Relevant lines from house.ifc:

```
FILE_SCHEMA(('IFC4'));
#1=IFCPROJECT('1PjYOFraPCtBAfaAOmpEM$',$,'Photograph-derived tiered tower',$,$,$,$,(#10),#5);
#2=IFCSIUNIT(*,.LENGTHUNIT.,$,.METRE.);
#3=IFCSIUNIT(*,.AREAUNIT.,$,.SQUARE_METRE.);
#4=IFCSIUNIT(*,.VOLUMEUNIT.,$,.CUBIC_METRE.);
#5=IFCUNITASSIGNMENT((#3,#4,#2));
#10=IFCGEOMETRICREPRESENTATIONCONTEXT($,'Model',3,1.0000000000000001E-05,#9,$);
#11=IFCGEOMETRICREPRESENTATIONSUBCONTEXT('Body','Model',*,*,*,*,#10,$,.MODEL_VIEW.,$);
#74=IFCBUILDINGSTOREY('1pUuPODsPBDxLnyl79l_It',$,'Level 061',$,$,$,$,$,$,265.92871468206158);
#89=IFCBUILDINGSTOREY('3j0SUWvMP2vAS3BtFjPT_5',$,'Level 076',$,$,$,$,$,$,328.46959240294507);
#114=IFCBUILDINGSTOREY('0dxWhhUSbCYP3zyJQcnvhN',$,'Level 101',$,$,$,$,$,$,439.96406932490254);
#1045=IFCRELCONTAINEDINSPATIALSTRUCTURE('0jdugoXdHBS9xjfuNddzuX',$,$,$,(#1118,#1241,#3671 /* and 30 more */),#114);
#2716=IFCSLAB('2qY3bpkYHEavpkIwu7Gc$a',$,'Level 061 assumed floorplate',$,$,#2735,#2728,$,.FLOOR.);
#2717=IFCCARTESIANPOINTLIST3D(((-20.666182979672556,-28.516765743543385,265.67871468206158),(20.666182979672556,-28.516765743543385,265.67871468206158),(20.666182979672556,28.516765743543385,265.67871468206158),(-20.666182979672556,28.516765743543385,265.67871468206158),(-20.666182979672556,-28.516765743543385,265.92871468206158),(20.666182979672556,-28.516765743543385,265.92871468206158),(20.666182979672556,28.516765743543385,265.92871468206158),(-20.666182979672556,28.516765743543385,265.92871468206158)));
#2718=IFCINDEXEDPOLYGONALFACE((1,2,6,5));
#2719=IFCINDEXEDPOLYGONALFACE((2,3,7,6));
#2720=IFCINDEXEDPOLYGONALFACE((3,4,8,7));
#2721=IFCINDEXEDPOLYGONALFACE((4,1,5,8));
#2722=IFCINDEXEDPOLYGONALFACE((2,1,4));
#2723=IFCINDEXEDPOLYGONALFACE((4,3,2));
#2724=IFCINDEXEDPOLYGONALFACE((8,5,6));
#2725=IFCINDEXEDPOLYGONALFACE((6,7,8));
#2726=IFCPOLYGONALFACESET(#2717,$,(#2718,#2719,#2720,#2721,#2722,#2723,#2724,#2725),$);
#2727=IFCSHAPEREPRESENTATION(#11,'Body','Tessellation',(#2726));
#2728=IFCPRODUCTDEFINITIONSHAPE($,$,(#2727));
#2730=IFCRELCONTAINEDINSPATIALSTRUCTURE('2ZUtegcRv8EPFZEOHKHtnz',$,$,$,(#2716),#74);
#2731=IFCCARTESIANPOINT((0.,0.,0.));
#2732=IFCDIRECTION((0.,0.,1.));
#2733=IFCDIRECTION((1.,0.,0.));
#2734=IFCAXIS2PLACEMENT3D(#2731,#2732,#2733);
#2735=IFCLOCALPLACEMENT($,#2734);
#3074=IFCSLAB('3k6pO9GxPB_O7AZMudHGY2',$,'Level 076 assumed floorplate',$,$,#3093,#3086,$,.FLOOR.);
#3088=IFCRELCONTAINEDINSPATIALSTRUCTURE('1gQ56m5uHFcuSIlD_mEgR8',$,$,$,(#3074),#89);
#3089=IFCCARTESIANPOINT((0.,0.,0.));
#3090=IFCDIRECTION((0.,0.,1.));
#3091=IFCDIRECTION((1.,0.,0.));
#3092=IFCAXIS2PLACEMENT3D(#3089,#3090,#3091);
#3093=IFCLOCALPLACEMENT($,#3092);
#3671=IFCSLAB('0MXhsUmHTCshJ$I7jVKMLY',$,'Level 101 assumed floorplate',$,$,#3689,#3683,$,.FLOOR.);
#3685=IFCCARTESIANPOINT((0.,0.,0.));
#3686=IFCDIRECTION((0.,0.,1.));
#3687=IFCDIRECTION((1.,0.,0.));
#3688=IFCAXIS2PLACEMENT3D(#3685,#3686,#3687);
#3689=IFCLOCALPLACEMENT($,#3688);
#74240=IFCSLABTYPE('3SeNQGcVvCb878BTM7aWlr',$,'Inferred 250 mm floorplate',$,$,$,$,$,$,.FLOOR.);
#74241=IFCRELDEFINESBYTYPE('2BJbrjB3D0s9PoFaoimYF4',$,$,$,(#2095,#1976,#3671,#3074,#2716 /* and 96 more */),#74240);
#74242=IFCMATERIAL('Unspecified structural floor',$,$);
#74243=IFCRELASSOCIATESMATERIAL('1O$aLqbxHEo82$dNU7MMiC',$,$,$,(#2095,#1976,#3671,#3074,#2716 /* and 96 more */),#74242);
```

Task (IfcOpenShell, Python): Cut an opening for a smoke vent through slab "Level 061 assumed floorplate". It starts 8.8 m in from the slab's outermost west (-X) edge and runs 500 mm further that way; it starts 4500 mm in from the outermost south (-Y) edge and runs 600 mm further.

```python
import numpy as np
import ifcopenshell
import ifcopenshell.api.feature
import ifcopenshell.api.geometry
import ifcopenshell.api.root
import ifcopenshell.geom
import ifcopenshell.util.placement
import ifcopenshell.util.representation
import ifcopenshell.util.shape
import ifcopenshell.util.unit

model = ifcopenshell.open("house.ifc")
unit_scale = ifcopenshell.util.unit.calculate_unit_scale(model)
settings = ifcopenshell.geom.settings()


def volume(element):
    """Net volume in cubic metres, openings subtracted."""
    shape = ifcopenshell.geom.create_shape(settings, element)
    return ifcopenshell.util.shape.get_volume(shape.geometry)


slab = model.by_id(2716)
before = volume(slab)

# Extent in the slab's own axes, in metres. The edges named are its -X and -Y sides.
slab_shape = ifcopenshell.geom.create_shape(settings, slab)
vertices = ifcopenshell.util.shape.get_vertices(slab_shape.geometry)
x_min, y_min, bottom = vertices.min(axis=0)
top = vertices[:, 2].max()

opening = ifcopenshell.api.root.create_entity(model, ifc_class="IfcOpeningElement", name="Smoke vent opening", predefined_type="OPENING")
context = ifcopenshell.util.representation.get_context(model, "Model", "Body", "MODEL_VIEW")
width, depth = 0.5, 0.6
outline = [(0.0, 0.0), (width, 0.0), (width, depth), (0.0, depth), (0.0, 0.0)]
# Overshoot both faces by 50 mm so the cut is clean.
shape = ifcopenshell.api.geometry.add_slab_representation(
    model, context=context, depth=top - bottom + 0.1, polyline=outline
)
ifcopenshell.api.geometry.assign_representation(model, product=opening, representation=shape)

matrix = ifcopenshell.util.placement.get_local_placement(slab.ObjectPlacement)
matrix[:, 3] = matrix @ np.append(np.array([x_min + 8.8, y_min + 4.5, bottom - 0.05]) / unit_scale, 1.0)
ifcopenshell.api.geometry.edit_object_placement(model, product=opening, matrix=matrix, is_si=False)
ifcopenshell.api.feature.add_feature(model, feature=opening, element=slab)

after = volume(slab)

print(f"slab volume {before:.3f} -> {after:.3f} m3")

model.write("house_rev.ifc")
```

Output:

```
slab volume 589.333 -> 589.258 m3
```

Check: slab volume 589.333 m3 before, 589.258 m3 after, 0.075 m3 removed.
